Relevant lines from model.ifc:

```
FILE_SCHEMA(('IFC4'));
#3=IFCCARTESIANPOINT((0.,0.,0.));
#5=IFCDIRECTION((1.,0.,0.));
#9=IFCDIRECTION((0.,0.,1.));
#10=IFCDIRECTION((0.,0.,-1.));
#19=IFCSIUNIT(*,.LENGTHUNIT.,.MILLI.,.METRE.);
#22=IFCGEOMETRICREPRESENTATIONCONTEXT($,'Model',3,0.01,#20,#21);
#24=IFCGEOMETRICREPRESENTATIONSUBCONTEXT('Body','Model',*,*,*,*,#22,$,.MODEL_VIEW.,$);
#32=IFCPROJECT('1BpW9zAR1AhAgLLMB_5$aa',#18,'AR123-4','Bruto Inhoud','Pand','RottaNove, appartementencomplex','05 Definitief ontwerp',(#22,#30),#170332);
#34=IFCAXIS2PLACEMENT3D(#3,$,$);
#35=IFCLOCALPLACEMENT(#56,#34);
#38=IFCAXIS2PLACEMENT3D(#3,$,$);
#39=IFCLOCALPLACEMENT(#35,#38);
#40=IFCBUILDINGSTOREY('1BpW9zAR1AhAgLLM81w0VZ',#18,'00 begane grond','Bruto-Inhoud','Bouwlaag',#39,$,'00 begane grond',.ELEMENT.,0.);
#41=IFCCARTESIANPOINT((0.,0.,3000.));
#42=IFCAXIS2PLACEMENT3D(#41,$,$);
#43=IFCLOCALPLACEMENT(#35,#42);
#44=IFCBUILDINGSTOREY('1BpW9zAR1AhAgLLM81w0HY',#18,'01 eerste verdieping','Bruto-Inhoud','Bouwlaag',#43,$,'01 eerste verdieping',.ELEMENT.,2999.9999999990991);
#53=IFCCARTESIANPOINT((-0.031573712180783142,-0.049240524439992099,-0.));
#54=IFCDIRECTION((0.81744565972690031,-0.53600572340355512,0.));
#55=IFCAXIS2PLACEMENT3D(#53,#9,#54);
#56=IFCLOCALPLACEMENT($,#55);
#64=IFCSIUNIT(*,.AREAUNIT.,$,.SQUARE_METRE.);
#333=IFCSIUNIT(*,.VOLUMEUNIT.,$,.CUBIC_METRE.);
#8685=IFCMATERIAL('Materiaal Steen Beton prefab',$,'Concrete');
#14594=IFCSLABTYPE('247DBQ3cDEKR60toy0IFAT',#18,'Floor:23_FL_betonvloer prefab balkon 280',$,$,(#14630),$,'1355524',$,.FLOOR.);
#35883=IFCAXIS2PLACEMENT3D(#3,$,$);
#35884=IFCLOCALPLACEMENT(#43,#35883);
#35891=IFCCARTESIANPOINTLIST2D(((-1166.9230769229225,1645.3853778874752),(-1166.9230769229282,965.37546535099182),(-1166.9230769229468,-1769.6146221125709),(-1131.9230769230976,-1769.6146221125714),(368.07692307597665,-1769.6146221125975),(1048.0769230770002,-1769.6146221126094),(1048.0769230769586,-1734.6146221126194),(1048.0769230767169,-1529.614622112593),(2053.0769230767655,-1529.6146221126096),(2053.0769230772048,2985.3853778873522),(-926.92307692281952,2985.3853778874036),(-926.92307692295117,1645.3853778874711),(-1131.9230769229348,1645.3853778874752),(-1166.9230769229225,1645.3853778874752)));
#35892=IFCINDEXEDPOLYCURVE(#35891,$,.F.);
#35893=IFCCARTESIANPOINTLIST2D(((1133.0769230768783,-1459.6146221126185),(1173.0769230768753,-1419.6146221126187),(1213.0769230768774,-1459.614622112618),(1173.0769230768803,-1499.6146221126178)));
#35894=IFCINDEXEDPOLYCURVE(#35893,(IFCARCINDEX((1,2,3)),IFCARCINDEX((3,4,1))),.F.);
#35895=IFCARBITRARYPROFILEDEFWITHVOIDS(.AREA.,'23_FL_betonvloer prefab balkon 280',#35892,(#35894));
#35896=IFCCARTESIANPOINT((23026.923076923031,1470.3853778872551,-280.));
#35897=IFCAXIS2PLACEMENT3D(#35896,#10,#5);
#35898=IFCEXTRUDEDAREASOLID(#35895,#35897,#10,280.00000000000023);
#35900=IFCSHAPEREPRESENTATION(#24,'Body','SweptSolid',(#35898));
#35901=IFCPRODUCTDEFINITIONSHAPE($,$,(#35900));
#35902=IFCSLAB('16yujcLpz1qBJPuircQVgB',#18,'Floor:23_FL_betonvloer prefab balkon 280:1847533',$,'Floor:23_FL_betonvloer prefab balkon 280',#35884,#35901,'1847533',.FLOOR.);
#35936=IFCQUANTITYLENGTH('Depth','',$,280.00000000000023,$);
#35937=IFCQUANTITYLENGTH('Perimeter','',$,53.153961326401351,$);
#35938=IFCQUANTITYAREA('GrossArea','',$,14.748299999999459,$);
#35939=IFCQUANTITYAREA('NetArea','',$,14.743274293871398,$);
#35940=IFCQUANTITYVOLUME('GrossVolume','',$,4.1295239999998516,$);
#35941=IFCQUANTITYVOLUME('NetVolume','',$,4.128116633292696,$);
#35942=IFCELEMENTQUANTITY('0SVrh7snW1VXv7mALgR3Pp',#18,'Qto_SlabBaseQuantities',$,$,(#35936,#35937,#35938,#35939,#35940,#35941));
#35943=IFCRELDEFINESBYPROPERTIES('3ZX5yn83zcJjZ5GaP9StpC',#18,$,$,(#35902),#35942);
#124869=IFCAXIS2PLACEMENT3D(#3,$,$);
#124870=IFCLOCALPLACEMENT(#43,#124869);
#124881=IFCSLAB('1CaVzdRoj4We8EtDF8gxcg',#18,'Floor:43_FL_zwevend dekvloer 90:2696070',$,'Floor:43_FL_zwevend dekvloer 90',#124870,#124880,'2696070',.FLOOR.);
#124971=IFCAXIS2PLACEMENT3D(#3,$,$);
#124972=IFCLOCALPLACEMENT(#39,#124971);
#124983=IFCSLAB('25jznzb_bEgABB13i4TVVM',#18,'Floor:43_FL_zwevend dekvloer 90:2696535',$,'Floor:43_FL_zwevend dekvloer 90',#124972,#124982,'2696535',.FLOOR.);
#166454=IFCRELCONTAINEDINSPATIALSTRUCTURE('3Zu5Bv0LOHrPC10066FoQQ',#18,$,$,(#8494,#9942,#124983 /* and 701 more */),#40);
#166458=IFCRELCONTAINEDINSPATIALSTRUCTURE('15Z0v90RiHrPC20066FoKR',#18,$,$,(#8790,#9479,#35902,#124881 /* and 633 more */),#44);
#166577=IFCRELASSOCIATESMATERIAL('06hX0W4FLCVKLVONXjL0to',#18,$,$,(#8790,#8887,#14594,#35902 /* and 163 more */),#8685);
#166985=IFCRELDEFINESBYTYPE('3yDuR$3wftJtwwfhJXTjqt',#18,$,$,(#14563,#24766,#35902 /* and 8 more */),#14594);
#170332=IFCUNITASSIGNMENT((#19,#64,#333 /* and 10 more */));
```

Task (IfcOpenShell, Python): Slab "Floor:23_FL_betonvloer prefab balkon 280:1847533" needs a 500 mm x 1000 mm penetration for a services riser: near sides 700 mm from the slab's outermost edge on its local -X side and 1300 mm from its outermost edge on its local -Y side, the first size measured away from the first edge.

```python
import numpy as np
import ifcopenshell
import ifcopenshell.api.feature
import ifcopenshell.api.geometry
import ifcopenshell.api.pset
import ifcopenshell.api.root
import ifcopenshell.geom
import ifcopenshell.util.element
import ifcopenshell.util.placement
import ifcopenshell.util.representation
import ifcopenshell.util.shape
import ifcopenshell.util.unit

model = ifcopenshell.open("model.ifc")
unit_scale = ifcopenshell.util.unit.calculate_unit_scale(model)
area_scale = ifcopenshell.util.unit.calculate_unit_scale(model, "AREAUNIT")
volume_scale = ifcopenshell.util.unit.calculate_unit_scale(model, "VOLUMEUNIT")
settings = ifcopenshell.geom.settings()


def volume(element):
    """Net volume in cubic metres, openings subtracted."""
    shape = ifcopenshell.geom.create_shape(settings, element)
    return ifcopenshell.util.shape.get_volume(shape.geometry)


slab = model.by_guid("16yujcLpz1qBJPuircQVgB")
before = volume(slab)

# Extent in the slab's own axes, in metres. The edges named are its -X and -Y sides.
slab_shape = ifcopenshell.geom.create_shape(settings, slab)
vertices = ifcopenshell.util.shape.get_vertices(slab_shape.geometry)
x_min, y_min, bottom = vertices.min(axis=0)
top = vertices[:, 2].max()

opening = ifcopenshell.api.root.create_entity(model, ifc_class="IfcOpeningElement", name="Services riser opening", predefined_type="OPENING")
context = ifcopenshell.util.representation.get_context(model, "Model", "Body", "MODEL_VIEW")
width, depth = 0.5, 1
outline = [(0.0, 0.0), (width, 0.0), (width, depth), (0.0, depth), (0.0, 0.0)]
# Overshoot both faces by 50 mm so the cut is clean.
shape = ifcopenshell.api.geometry.add_slab_representation(
    model, context=context, depth=top - bottom + 0.1, polyline=outline
)
ifcopenshell.api.geometry.assign_representation(model, product=opening, representation=shape)

matrix = ifcopenshell.util.placement.get_local_placement(slab.ObjectPlacement)
matrix[:, 3] = matrix @ np.append(np.array([x_min + 0.7, y_min + 1.3, bottom - 0.05]) / unit_scale, 1.0)
ifcopenshell.api.geometry.edit_object_placement(model, product=opening, matrix=matrix, is_si=False)
ifcopenshell.api.feature.add_feature(model, feature=opening, element=slab)

after = volume(slab)

# Update the slab's stored quantities.
qto = model.by_id(ifcopenshell.util.element.get_pset(slab, "Qto_SlabBaseQuantities", should_inherit=False)["id"])
ifcopenshell.api.pset.edit_qto(model, qto=qto, properties={
    "NetArea": after / (top - bottom) / area_scale,
    "NetVolume": after / volume_scale,
})

print(f"slab volume {before:.3f} -> {after:.3f} m3")

model.write("model_updated.ifc")
```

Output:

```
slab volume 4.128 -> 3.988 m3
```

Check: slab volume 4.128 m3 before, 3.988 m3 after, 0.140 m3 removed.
